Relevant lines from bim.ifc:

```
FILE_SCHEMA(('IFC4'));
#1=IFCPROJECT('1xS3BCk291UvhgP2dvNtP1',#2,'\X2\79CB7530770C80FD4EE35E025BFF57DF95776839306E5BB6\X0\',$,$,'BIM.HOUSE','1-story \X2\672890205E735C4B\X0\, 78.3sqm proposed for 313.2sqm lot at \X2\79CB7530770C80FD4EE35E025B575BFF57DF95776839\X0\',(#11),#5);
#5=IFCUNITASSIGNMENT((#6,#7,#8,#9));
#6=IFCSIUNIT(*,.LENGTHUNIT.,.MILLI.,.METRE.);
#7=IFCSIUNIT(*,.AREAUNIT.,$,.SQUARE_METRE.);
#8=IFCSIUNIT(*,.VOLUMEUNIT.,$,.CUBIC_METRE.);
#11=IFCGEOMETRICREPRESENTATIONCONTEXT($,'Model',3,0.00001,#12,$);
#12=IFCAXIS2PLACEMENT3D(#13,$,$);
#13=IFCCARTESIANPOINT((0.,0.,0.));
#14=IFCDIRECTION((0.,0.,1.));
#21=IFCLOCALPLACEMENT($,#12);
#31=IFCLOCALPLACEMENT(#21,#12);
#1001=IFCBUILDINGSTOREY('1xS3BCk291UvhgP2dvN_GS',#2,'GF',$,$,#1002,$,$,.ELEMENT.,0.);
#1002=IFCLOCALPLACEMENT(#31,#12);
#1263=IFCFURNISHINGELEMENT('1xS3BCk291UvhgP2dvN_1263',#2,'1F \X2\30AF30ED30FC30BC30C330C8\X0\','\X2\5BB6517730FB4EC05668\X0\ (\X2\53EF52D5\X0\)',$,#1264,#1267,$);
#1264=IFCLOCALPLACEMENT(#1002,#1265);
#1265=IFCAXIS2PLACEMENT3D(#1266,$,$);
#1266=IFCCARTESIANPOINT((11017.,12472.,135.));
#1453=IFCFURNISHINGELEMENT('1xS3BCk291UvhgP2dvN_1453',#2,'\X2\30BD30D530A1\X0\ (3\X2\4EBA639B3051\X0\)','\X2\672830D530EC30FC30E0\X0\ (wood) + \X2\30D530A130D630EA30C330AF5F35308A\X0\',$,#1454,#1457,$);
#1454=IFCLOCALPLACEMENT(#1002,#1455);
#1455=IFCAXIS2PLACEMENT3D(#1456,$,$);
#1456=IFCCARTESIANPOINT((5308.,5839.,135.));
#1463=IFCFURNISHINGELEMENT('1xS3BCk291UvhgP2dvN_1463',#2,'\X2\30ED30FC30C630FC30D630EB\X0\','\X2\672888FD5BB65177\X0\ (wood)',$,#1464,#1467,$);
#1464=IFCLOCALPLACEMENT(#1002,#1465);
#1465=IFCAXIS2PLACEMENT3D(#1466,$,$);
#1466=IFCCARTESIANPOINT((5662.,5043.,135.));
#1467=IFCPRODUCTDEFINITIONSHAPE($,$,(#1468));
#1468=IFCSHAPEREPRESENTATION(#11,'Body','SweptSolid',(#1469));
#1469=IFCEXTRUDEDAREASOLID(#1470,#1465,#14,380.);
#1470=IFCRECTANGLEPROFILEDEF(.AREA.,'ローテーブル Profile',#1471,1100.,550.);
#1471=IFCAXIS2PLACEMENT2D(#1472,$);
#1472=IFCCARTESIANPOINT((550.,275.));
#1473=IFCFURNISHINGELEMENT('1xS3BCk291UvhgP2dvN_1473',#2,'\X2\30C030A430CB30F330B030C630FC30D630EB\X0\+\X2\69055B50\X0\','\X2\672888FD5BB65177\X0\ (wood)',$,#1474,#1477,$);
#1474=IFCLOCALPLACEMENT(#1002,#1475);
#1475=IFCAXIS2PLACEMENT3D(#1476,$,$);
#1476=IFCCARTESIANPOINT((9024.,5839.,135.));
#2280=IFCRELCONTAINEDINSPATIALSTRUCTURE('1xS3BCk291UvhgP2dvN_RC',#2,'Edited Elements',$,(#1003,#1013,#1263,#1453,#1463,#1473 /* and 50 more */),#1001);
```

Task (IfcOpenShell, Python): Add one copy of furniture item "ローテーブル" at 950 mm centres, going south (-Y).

```python
import numpy as np
import ifcopenshell
import ifcopenshell.api.geometry
import ifcopenshell.api.root
import ifcopenshell.util.element
import ifcopenshell.util.placement

model = ifcopenshell.open("bim.ifc")


def reuse_history(source, copy):
    """copy_class also copies each property set's owner history, people and application; keep the originals."""
    for rel in copy.IsDefinedBy:
        if rel.is_a("IfcRelDefinesByProperties") and (history := rel.RelatingPropertyDefinition.OwnerHistory):
            rel.RelatingPropertyDefinition.OwnerHistory = source.OwnerHistory
            ifcopenshell.util.element.remove_deep2(model, history)


source = model.by_id(1463)
base = ifcopenshell.util.placement.get_local_placement(source.ObjectPlacement)
step = np.array([0.0, -1.0, 0.0]) * 950.0

for i in range(1, 2):
    copy = ifcopenshell.api.root.copy_class(model, product=source)
    copy.Representation = ifcopenshell.util.element.copy_deep(
        model, source.Representation, exclude=["IfcGeometricRepresentationContext", "IfcRepresentationMap"]
    )
    reuse_history(source, copy)
    matrix = base.copy()
    matrix[:3, 3] += i * step
    print("added at", matrix[:3, 3].round(3) + 0.0)
    ifcopenshell.api.geometry.edit_object_placement(model, product=copy, matrix=matrix, is_si=False)

model.write("bim_edited.ifc")
```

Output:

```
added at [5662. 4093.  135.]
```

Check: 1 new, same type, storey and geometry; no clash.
